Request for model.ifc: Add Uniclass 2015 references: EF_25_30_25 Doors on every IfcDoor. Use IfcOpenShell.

First a look at what the model holds.

```python
import ifcopenshell

model = ifcopenshell.open("model.ifc")
print(model.schema)
print("classifications:", [c.Name for c in model.by_type("IfcClassification")])
for ifc_class in ("IfcDoor", "IfcRoof", "IfcStair", "IfcWall", "IfcWindow"):
    print(ifc_class, len(model.by_type(ifc_class)))
```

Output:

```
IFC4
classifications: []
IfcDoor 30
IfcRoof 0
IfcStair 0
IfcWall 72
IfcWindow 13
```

```python
import ifcopenshell
import ifcopenshell.api.classification

model = ifcopenshell.open("model.ifc")

system = ifcopenshell.api.classification.add_classification(model, classification="Uniclass 2015")

codes = {
    "IfcDoor": ("EF_25_30_25", "Doors"),
}
for ifc_class, (code, name) in codes.items():
    products = model.by_type(ifc_class)
    ifcopenshell.api.classification.add_reference(
        model, products=products, classification=system, identification=code, name=name
    )
    print(code, len(products))

model.write("model_rev.ifc")
```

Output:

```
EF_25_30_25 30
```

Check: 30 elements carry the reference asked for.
